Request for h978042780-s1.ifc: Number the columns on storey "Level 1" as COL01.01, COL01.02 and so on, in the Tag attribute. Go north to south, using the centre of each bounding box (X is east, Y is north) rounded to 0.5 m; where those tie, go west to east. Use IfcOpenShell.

First a look at what the model holds.

```python
import ifcopenshell
import ifcopenshell.util.element
import ifcopenshell.util.placement

model = ifcopenshell.open("h978042780-s1.ifc")
print(model.schema)
storey = next(s for s in model.by_type("IfcBuildingStorey") if s.Name == "Level 1")
columns = [e for e in ifcopenshell.util.element.get_decomposition(storey) if e.is_a("IfcColumn")]
for e in sorted(columns, key=lambda e: e.id()):
    origin = ifcopenshell.util.placement.get_local_placement(e.ObjectPlacement)[:3, 3]
    print(e.id(), e.Tag, e.Name, origin.round(2) + 0.0, sep=" | ")
```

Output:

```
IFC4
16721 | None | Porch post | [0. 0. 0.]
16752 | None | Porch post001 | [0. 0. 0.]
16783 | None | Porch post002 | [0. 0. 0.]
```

```python
import ifcopenshell
import ifcopenshell.geom
import ifcopenshell.util.element
import ifcopenshell.util.shape

model = ifcopenshell.open("h978042780-s1.ifc")
settings = ifcopenshell.geom.settings()
settings.set("use-world-coords", True)


def centre(element):
    shape = ifcopenshell.geom.create_shape(settings, element)
    return ifcopenshell.util.shape.get_bbox_centroid(shape.geometry)


storey = next(s for s in model.by_type("IfcBuildingStorey") if s.Name == "Level 1")
columns = [e for e in ifcopenshell.util.element.get_decomposition(storey) if e.is_a("IfcColumn")]

# Insertion points can sit at a corner or the storey origin, so sort by the geometry (in metres).
centres = {e: centre(e) for e in columns}
columns.sort(key=lambda e: (-round(centres[e][1] / 0.5), centres[e][0]))

for i, e in enumerate(columns, start=1):
    number = f"COL01.{i:02d}"
    e.Tag = number
    print(e.id(), number)

model.write("h978042780-s1_updated.ifc")
```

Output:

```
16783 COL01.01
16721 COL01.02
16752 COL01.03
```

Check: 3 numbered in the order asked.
